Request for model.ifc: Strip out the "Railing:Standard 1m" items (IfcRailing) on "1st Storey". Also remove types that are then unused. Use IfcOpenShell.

First a look at what the model holds.

```python
import ifcopenshell
import ifcopenshell.util.element

model = ifcopenshell.open("model.ifc")
print(model.schema)
storey = next(s for s in model.by_type("IfcBuildingStorey") if s.Name == "1st Storey")
railings = [e for e in ifcopenshell.util.element.get_decomposition(storey) if e.is_a("IfcRailing")]
seen = {}
for e in railings:
    element_type = ifcopenshell.util.element.get_type(e)
    name = element_type.Name if element_type not in (None, e) else None
    seen[name] = seen.get(name, 0) + 1
for name, count in sorted(seen.items(), key=str):
    print(count, "x", name)
```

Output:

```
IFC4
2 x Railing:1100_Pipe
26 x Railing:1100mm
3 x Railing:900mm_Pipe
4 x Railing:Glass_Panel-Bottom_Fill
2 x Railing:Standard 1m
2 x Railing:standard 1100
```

```python
import ifcopenshell
import ifcopenshell.api.root
import ifcopenshell.util.element

model = ifcopenshell.open("model.ifc")

storey = next(s for s in model.by_type("IfcBuildingStorey") if s.Name == "1st Storey")
railings = [e for e in ifcopenshell.util.element.get_decomposition(storey) if e.is_a("IfcRailing")]
targets = [e for e in railings if (t := ifcopenshell.util.element.get_type(e)) not in (None, e) and t.Name == "Railing:Standard 1m"]
types = {ifcopenshell.util.element.get_type(e) for e in targets} - {None, *targets}

for e in targets:
    ifcopenshell.api.root.remove_product(model, product=e)
print(len(targets), "removed")

unused = [t for t in types if not ifcopenshell.util.element.get_types(t)]
for t in unused:
    ifcopenshell.api.root.remove_product(model, product=t)
print(len(unused), "unused types removed")

model.write("model_v2.ifc")
```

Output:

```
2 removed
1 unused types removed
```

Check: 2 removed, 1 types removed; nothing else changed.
